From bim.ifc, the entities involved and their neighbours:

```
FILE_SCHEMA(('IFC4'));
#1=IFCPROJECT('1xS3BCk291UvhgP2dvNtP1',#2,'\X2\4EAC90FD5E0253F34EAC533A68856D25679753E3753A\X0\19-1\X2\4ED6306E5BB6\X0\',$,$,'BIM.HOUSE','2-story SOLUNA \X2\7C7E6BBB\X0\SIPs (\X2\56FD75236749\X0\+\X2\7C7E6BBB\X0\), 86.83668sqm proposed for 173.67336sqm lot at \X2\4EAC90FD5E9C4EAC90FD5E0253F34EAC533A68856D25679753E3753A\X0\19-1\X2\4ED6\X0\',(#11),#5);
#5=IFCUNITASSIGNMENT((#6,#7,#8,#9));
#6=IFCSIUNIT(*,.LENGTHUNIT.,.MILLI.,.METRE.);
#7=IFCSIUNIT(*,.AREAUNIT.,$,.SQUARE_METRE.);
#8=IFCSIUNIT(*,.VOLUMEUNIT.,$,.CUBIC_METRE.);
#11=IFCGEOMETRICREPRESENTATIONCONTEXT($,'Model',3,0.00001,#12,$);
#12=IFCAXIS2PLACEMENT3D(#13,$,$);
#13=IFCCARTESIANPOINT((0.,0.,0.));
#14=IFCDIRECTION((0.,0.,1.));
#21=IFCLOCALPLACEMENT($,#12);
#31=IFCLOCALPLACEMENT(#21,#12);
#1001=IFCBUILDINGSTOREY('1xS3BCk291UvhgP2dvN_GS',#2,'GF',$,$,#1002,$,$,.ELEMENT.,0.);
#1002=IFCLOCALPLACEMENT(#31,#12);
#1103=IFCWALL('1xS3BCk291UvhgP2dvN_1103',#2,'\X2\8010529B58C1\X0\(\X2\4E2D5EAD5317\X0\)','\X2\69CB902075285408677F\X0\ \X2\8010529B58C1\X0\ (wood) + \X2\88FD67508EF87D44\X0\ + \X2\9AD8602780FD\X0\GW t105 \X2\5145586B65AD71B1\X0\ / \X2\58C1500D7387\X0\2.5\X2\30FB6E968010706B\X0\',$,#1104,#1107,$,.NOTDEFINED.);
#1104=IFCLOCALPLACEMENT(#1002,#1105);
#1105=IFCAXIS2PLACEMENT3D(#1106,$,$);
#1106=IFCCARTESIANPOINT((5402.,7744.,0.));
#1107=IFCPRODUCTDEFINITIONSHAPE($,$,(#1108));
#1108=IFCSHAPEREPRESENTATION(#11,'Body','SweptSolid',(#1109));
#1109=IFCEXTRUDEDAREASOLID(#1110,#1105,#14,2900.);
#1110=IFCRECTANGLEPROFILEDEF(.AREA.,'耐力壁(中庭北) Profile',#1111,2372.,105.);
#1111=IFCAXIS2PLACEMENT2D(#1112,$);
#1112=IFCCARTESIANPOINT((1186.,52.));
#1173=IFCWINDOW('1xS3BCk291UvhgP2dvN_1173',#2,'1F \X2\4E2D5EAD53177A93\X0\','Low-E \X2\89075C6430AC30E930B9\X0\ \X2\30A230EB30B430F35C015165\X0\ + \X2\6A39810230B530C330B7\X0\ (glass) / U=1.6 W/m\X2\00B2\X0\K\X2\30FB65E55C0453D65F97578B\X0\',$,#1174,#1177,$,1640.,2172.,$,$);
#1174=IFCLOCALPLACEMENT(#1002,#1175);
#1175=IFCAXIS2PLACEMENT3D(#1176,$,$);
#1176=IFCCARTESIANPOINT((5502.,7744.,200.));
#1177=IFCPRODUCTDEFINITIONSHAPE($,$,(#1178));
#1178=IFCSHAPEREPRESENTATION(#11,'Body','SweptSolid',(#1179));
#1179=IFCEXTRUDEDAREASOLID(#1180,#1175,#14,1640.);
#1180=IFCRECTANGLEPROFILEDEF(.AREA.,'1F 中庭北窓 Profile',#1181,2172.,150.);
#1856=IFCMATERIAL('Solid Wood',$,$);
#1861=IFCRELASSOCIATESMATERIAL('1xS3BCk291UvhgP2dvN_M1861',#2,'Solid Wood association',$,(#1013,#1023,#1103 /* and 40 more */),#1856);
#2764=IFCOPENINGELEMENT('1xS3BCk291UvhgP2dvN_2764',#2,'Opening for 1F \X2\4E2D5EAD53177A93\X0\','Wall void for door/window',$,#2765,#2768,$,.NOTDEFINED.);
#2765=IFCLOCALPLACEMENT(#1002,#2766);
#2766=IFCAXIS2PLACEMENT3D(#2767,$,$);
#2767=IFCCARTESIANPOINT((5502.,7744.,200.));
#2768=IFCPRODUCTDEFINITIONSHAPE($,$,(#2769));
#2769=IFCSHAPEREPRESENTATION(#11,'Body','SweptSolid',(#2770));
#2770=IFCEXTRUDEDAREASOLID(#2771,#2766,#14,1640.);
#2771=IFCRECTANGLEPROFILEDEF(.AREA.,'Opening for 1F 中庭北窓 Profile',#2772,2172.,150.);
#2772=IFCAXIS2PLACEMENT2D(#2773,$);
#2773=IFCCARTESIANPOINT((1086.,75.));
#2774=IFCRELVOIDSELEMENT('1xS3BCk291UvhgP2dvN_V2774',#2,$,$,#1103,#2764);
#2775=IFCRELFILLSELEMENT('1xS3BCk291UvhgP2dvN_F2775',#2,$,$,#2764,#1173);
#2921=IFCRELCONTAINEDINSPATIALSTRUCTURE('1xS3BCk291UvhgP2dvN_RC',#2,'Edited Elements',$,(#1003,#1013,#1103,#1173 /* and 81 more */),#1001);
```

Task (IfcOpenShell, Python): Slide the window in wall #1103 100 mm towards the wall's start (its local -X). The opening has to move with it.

```python
import ifcopenshell
import ifcopenshell.api.geometry
import ifcopenshell.util.placement
import ifcopenshell.util.unit

model = ifcopenshell.open("bim.ifc")
unit_scale = ifcopenshell.util.unit.calculate_unit_scale(model)

window = model.by_guid("1xS3BCk291UvhgP2dvN_1173")
opening = window.FillsVoids[0].RelatingOpeningElement
wall = opening.VoidsElements[0].RelatingBuildingElement

wall_matrix = ifcopenshell.util.placement.get_local_placement(wall.ObjectPlacement)
shift = wall_matrix[:3, 0] * -0.1 / unit_scale
before = ifcopenshell.util.placement.get_local_placement(window.ObjectPlacement)[:3, 3].copy()

# The window is not placed relative to its opening, so move both.
for product in (opening, window):
    matrix = ifcopenshell.util.placement.get_local_placement(product.ObjectPlacement)
    matrix[:3, 3] += shift
    ifcopenshell.api.geometry.edit_object_placement(model, product=product, matrix=matrix, is_si=False)

after = ifcopenshell.util.placement.get_local_placement(window.ObjectPlacement)[:3, 3]
print("window moved by", (after - before).round(3) + 0.0)

model.write("bim_edited.ifc")
```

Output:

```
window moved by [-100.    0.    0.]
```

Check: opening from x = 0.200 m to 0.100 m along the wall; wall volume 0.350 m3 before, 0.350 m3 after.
